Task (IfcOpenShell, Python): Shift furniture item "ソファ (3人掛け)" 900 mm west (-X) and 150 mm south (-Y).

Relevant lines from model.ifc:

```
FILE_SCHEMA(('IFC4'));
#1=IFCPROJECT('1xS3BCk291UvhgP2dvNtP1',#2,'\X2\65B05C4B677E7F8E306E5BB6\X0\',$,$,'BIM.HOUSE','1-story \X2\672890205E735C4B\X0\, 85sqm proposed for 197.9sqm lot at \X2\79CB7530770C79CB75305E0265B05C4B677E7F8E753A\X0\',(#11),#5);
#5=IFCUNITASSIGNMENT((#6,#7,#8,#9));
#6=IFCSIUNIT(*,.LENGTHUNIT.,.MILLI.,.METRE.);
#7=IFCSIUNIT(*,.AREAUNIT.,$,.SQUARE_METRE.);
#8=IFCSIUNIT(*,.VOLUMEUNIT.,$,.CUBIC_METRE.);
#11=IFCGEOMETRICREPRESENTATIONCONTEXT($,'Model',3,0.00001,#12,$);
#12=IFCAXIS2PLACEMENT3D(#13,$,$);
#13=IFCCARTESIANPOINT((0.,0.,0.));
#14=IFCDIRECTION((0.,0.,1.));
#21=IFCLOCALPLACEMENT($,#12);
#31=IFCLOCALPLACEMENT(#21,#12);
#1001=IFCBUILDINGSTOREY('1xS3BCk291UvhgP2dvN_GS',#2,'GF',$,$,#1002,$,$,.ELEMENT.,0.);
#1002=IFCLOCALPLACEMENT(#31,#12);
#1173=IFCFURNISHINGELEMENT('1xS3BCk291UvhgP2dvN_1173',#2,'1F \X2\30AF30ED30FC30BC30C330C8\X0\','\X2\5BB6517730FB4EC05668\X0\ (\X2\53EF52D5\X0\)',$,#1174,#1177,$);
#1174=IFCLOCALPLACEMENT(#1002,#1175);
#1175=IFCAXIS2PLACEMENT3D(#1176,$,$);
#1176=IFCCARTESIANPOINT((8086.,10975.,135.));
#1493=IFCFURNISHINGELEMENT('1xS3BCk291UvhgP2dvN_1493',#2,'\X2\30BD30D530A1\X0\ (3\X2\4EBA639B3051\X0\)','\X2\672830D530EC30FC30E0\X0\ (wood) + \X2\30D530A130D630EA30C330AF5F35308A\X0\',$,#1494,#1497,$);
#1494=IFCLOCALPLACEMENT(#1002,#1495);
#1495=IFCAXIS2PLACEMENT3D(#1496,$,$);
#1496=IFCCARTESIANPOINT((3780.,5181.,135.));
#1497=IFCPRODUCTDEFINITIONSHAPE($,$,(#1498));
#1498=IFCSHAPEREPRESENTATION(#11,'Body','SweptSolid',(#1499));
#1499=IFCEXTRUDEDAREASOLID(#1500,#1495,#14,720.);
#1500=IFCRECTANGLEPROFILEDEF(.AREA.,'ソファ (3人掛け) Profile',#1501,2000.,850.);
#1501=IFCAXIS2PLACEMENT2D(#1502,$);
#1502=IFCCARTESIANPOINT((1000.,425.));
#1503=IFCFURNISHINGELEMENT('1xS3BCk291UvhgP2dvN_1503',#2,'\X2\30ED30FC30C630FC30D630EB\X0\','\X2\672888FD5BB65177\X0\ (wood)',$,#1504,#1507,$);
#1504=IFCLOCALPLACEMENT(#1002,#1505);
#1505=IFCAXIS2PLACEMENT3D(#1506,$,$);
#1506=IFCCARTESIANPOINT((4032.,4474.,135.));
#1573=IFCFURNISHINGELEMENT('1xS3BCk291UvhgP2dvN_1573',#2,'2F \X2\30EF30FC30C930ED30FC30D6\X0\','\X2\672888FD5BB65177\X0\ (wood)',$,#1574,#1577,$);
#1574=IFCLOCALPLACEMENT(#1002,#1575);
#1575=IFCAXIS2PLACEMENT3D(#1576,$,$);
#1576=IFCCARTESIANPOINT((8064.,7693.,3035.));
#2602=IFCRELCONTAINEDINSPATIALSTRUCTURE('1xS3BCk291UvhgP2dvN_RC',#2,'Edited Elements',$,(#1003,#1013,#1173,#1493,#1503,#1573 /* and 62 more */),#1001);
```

```python
import ifcopenshell
import ifcopenshell.api.geometry
import ifcopenshell.util.placement

model = ifcopenshell.open("model.ifc")

item = model.by_id(1493)
matrix = ifcopenshell.util.placement.get_local_placement(item.ObjectPlacement)
matrix[0, 3] -= 900.0
matrix[1, 3] -= 150.0
ifcopenshell.api.geometry.edit_object_placement(model, product=item, matrix=matrix, is_si=False)

print(ifcopenshell.util.placement.get_local_placement(item.ObjectPlacement).round(3) + 0.0)

model.write("model-out.ifc")
```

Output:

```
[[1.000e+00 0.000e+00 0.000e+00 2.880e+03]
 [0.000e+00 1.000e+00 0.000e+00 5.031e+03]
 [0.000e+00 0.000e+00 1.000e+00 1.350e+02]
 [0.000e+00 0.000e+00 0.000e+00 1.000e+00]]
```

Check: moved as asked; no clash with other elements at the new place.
